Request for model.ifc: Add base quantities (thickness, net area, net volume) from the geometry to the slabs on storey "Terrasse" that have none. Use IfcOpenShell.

First a look at what the model holds.

```python
import ifcopenshell
import ifcopenshell.util.element
import ifcopenshell.util.unit

model = ifcopenshell.open("model.ifc")
print(model.schema)
for unit_type in ("LENGTHUNIT", "AREAUNIT", "VOLUMEUNIT"):
    print(unit_type, ifcopenshell.util.unit.calculate_unit_scale(model, unit_type))
storey = next(s for s in model.by_type("IfcBuildingStorey") if s.Name == "Terrasse")
slabs = [e for e in ifcopenshell.util.element.get_decomposition(storey) if e.is_a("IfcSlab")]
for e in sorted(slabs, key=lambda e: e.id()):
    print(e.id(), e.is_a(), e.Name, list(ifcopenshell.util.element.get_psets(e, qtos_only=True)), sep=" | ")
```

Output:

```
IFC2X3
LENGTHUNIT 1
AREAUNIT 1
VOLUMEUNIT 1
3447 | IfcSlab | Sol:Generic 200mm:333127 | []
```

```python
import ifcopenshell
import ifcopenshell.api.pset
import ifcopenshell.geom
import ifcopenshell.util.element
import ifcopenshell.util.shape
import ifcopenshell.util.unit

model = ifcopenshell.open("model.ifc")
unit_scale = ifcopenshell.util.unit.calculate_unit_scale(model)
area_scale = ifcopenshell.util.unit.calculate_unit_scale(model, "AREAUNIT")
volume_scale = ifcopenshell.util.unit.calculate_unit_scale(model, "VOLUMEUNIT")
settings = ifcopenshell.geom.settings()

storey = next(s for s in model.by_type("IfcBuildingStorey") if s.Name == "Terrasse")
slabs = [e for e in ifcopenshell.util.element.get_decomposition(storey) if e.is_a("IfcSlab")]

for e in sorted(slabs, key=lambda e: e.id()):
    if ifcopenshell.util.element.get_psets(e, qtos_only=True, should_inherit=False):
        continue
    # Geometry comes back in metres, in the element's own axes.
    shape = ifcopenshell.geom.create_shape(settings, e)
    values = {
        "Width": ifcopenshell.util.shape.get_z(shape.geometry) / unit_scale,
        "NetArea": ifcopenshell.util.shape.get_footprint_area(shape.geometry) / area_scale,
        "NetVolume": ifcopenshell.util.shape.get_volume(shape.geometry) / volume_scale,
    }
    qto = ifcopenshell.api.pset.add_qto(model, product=e, name="BaseQuantities")
    ifcopenshell.api.pset.edit_qto(model, qto=qto, properties=values)
    print(e.id(), {k: round(v, 3) for k, v in values.items()})

model.write("model_rev.ifc")
```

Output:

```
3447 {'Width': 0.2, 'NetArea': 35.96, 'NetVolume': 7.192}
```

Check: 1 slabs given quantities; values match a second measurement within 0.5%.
